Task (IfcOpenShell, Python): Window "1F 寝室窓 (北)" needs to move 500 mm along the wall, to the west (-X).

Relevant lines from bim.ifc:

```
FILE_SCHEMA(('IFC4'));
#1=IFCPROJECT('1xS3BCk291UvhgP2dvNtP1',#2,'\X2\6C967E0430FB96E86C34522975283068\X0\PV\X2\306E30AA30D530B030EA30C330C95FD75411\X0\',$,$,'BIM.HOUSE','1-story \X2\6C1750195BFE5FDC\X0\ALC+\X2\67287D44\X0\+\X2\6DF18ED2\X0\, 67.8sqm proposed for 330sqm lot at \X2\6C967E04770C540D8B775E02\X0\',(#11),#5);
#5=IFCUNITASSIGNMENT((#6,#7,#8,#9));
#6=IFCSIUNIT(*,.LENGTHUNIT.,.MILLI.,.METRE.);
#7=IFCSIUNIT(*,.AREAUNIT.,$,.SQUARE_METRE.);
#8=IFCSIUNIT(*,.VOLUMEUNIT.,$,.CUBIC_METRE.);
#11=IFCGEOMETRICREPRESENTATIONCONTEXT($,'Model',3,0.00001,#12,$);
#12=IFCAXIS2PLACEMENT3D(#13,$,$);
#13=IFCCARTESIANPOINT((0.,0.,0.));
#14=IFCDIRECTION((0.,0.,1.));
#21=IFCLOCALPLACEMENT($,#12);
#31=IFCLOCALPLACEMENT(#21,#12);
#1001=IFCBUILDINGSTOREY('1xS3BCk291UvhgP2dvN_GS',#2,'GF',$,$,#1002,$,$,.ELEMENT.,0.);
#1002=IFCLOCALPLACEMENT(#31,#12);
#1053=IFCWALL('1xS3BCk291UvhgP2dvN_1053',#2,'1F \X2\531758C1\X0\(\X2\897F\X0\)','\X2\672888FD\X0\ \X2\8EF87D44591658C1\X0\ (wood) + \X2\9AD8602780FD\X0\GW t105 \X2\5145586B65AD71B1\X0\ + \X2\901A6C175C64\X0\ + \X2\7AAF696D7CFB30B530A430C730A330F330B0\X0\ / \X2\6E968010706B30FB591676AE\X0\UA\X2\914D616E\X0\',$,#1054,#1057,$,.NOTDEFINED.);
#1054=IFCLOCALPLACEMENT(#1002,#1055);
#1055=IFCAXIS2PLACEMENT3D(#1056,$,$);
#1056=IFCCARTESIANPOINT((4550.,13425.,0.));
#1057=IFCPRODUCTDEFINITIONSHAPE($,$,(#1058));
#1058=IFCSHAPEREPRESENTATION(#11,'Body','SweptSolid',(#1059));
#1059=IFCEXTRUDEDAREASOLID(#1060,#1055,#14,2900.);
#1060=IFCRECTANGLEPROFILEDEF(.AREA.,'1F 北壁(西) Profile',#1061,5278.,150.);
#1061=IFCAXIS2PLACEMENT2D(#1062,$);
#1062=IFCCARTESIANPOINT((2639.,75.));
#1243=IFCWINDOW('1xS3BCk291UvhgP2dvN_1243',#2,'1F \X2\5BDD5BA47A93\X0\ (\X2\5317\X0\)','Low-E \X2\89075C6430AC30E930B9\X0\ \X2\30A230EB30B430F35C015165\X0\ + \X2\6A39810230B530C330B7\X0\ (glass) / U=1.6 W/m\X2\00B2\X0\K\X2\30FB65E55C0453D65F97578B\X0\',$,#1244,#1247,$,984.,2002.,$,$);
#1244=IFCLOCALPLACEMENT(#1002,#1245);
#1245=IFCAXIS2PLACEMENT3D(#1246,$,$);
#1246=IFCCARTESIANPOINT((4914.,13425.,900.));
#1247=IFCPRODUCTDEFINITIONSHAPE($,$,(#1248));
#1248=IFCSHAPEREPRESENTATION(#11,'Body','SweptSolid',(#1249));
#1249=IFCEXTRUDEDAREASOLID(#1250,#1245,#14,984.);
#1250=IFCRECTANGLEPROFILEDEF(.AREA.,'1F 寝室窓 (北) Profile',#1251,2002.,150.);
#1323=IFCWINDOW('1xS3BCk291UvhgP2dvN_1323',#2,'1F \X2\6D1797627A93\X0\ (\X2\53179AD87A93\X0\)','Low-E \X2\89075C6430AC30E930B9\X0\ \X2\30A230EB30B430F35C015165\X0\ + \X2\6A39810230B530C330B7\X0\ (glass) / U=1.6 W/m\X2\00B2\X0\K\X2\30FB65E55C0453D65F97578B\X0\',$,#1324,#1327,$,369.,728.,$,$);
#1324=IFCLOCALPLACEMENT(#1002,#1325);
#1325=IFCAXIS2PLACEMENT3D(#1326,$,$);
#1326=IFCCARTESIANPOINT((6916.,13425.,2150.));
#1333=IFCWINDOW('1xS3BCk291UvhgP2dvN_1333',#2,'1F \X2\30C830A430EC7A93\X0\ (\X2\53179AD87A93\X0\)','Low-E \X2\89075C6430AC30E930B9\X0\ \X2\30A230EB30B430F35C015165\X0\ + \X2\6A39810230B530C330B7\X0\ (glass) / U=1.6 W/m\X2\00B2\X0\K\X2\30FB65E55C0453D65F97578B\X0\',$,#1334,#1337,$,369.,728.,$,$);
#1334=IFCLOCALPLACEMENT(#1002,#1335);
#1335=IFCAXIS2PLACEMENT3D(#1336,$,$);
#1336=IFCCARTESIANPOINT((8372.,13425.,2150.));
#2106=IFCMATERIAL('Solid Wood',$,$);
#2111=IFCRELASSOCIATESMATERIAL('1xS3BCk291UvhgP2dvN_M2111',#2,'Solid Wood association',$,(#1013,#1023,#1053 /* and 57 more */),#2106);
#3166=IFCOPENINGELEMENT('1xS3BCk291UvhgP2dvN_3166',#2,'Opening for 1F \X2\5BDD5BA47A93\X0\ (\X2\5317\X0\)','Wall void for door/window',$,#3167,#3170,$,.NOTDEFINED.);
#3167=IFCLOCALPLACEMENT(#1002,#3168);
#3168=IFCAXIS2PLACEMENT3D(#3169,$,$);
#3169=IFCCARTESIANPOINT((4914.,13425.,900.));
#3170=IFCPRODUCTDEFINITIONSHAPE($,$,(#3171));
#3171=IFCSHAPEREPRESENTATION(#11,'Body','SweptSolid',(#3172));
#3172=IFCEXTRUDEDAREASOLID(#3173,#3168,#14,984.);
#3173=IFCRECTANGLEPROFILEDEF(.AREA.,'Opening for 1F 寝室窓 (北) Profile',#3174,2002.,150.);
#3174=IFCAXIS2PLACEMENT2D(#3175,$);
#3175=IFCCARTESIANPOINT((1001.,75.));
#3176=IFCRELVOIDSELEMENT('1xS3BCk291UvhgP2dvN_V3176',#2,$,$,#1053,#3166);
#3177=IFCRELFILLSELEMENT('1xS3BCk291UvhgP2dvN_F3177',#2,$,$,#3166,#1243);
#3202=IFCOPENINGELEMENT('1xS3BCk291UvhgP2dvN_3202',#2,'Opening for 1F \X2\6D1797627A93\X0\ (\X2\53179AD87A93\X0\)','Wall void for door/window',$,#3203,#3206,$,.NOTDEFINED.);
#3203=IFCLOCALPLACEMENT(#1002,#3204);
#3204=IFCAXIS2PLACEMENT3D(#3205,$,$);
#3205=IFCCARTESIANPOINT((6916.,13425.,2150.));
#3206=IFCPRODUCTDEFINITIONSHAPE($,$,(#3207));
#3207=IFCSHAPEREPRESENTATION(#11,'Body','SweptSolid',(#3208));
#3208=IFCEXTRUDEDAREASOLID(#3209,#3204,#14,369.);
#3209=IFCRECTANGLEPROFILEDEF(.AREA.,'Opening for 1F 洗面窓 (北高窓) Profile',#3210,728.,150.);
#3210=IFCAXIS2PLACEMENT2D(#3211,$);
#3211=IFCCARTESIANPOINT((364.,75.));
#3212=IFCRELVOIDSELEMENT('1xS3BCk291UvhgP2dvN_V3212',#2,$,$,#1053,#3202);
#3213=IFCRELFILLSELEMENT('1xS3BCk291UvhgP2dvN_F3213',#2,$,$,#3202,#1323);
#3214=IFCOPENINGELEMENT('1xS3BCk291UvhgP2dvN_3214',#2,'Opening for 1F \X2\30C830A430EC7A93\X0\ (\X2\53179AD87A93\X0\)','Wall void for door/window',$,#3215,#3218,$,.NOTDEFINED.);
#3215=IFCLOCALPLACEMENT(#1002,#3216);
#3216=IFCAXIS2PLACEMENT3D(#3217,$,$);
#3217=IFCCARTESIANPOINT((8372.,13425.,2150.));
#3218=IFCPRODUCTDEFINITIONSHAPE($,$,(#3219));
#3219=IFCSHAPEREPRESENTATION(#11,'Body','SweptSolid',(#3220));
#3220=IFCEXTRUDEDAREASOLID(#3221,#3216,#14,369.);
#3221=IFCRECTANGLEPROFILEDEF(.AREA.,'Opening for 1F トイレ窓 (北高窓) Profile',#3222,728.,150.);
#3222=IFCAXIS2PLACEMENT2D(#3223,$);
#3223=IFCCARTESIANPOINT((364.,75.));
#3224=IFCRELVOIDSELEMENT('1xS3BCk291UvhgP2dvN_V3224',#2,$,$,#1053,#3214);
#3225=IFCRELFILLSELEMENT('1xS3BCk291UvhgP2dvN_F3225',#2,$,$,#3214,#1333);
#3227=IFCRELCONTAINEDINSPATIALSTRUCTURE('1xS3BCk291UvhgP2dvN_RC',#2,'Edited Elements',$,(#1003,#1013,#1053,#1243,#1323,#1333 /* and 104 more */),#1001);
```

```python
import ifcopenshell
import ifcopenshell.api.geometry
import ifcopenshell.util.placement

model = ifcopenshell.open("bim.ifc")

window = model.by_guid("1xS3BCk291UvhgP2dvN_1243")
opening = window.FillsVoids[0].RelatingOpeningElement
wall = opening.VoidsElements[0].RelatingBuildingElement

wall_matrix = ifcopenshell.util.placement.get_local_placement(wall.ObjectPlacement)
shift = wall_matrix[:3, 0] * -500.0
before = ifcopenshell.util.placement.get_local_placement(window.ObjectPlacement)[:3, 3].copy()

# The window is not placed relative to its opening, so move both.
for product in (opening, window):
    matrix = ifcopenshell.util.placement.get_local_placement(product.ObjectPlacement)
    matrix[:3, 3] += shift
    ifcopenshell.api.geometry.edit_object_placement(model, product=product, matrix=matrix, is_si=False)

after = ifcopenshell.util.placement.get_local_placement(window.ObjectPlacement)[:3, 3]
print("window moved by", (after - before).round(3) + 0.0)

model.write("bim_v2.ifc")
```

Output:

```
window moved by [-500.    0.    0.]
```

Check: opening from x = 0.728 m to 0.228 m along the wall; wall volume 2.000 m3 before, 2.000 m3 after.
